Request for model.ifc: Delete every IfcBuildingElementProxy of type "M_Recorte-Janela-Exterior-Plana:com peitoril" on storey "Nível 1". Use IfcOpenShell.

First a look at what the model holds.

```python
import ifcopenshell
import ifcopenshell.util.element

model = ifcopenshell.open("model.ifc")
print(model.schema)
storey = next(s for s in model.by_type("IfcBuildingStorey") if s.Name == "Nível 1")
proxies = [e for e in ifcopenshell.util.element.get_decomposition(storey) if e.is_a("IfcBuildingElementProxy")]
seen = {}
for e in proxies:
    element_type = ifcopenshell.util.element.get_type(e)
    name = element_type.Name if element_type not in (None, e) else None
    seen[name] = seen.get(name, 0) + 1
for name, count in sorted(seen.items(), key=str):
    print(count, "x", name)
```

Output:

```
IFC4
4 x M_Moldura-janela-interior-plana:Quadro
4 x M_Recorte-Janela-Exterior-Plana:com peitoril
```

```python
import ifcopenshell
import ifcopenshell.api.root
import ifcopenshell.util.element

model = ifcopenshell.open("model.ifc")

storey = next(s for s in model.by_type("IfcBuildingStorey") if s.Name == "Nível 1")
proxies = [e for e in ifcopenshell.util.element.get_decomposition(storey) if e.is_a("IfcBuildingElementProxy")]
targets = [e for e in proxies if (t := ifcopenshell.util.element.get_type(e)) not in (None, e) and t.Name == "M_Recorte-Janela-Exterior-Plana:com peitoril"]

for e in targets:
    ifcopenshell.api.root.remove_product(model, product=e)
print(len(targets), "removed")

model.write("model_edited.ifc")
```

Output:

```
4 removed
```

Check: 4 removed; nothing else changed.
